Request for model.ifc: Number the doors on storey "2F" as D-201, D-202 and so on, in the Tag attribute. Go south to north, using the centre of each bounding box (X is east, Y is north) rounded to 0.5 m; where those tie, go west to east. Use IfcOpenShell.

First a look at what the model holds.

```python
import ifcopenshell
import ifcopenshell.util.element
import ifcopenshell.util.placement

model = ifcopenshell.open("model.ifc")
print(model.schema)
storey = next(s for s in model.by_type("IfcBuildingStorey") if s.Name == "2F")
doors = [e for e in ifcopenshell.util.element.get_decomposition(storey) if e.is_a("IfcDoor")]
for e in sorted(doors, key=lambda e: e.id()):
    origin = ifcopenshell.util.placement.get_local_placement(e.ObjectPlacement)[:3, 3]
    print(e.id(), e.Tag, e.Name, origin.round(2) + 0.0, sep=" | ")
```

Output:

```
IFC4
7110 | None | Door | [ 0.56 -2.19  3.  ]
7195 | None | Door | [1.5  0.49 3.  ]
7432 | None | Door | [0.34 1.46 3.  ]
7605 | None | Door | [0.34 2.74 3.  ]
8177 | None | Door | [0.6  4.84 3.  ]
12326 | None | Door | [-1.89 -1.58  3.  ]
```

```python
import ifcopenshell
import ifcopenshell.geom
import ifcopenshell.util.element
import ifcopenshell.util.shape

model = ifcopenshell.open("model.ifc")
settings = ifcopenshell.geom.settings()
settings.set("use-world-coords", True)


def centre(element):
    shape = ifcopenshell.geom.create_shape(settings, element)
    return ifcopenshell.util.shape.get_bbox_centroid(shape.geometry)


storey = next(s for s in model.by_type("IfcBuildingStorey") if s.Name == "2F")
doors = [e for e in ifcopenshell.util.element.get_decomposition(storey) if e.is_a("IfcDoor")]

# Insertion points can sit at a corner or the storey origin, so sort by the geometry (in metres).
centres = {e: centre(e) for e in doors}
doors.sort(key=lambda e: (round(centres[e][1] / 0.5), centres[e][0]))

for i, e in enumerate(doors, start=1):
    number = f"D-2{i:02d}"
    e.Tag = number
    print(e.id(), number)

model.write("model_edited.ifc")
```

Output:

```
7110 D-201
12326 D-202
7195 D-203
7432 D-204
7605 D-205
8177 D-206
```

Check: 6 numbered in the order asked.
